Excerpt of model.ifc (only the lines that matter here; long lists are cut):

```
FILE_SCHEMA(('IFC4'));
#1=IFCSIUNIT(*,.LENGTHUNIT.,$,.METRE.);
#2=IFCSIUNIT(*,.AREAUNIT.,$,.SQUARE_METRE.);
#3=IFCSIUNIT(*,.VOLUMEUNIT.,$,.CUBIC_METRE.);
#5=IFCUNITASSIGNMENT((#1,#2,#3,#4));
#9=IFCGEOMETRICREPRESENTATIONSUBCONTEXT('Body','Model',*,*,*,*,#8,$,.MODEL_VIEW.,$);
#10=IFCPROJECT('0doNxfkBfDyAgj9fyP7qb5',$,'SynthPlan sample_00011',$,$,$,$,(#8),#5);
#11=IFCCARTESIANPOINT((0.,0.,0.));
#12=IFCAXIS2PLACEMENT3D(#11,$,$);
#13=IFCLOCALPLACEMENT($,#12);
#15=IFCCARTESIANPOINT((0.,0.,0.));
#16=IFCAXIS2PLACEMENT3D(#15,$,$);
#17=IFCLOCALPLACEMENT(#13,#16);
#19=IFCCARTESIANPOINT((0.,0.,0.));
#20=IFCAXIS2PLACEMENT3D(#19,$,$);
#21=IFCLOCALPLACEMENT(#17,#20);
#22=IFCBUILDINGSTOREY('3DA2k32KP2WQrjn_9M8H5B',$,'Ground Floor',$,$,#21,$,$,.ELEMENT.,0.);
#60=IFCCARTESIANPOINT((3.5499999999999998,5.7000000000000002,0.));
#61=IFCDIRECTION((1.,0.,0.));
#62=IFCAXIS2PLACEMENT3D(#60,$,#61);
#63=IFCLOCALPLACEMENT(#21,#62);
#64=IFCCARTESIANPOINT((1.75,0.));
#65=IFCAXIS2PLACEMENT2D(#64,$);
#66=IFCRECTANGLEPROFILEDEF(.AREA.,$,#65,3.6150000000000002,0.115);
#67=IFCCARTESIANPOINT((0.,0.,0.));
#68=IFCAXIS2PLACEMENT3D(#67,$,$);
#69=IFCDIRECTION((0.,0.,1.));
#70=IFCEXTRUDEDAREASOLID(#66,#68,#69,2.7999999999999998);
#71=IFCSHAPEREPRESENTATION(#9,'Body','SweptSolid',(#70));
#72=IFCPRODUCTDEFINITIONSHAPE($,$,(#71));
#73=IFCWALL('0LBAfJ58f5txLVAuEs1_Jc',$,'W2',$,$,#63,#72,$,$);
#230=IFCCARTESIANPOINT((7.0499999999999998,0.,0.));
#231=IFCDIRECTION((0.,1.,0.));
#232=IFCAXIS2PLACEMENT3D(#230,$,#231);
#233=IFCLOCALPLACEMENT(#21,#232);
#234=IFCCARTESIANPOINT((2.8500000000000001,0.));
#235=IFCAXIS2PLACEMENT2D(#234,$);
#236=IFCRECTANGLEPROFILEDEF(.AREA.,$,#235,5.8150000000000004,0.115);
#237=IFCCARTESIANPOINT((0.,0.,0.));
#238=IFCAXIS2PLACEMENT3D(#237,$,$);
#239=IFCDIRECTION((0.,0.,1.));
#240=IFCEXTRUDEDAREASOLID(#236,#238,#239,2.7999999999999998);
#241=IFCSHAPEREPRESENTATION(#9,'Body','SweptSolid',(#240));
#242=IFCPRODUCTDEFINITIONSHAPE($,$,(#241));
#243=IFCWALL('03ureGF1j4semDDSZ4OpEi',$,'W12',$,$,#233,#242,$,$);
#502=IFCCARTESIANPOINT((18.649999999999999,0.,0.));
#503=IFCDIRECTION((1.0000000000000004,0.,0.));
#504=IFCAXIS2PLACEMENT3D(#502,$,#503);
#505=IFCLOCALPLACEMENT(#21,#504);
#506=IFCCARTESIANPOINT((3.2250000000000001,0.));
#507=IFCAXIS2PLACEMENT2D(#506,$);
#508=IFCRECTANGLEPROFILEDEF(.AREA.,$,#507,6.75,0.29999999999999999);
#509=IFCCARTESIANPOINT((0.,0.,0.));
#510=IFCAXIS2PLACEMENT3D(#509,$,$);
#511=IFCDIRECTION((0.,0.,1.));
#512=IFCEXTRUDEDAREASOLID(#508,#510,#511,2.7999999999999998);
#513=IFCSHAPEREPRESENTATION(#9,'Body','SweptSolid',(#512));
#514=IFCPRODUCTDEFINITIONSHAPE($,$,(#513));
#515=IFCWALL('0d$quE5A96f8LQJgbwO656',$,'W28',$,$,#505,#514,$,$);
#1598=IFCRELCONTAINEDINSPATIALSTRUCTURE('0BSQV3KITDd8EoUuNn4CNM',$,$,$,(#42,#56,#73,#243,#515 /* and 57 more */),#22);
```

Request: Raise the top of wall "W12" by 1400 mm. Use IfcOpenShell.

```python
import ifcopenshell
import ifcopenshell.geom
import ifcopenshell.util.representation
import ifcopenshell.util.shape
import ifcopenshell.util.unit

model = ifcopenshell.open("model.ifc")
unit_scale = ifcopenshell.util.unit.calculate_unit_scale(model)
settings = ifcopenshell.geom.settings()


def volume(element):
    """Net volume in cubic metres, openings subtracted."""
    shape = ifcopenshell.geom.create_shape(settings, element)
    return ifcopenshell.util.shape.get_volume(shape.geometry)


wall = model.by_id(243)
before = volume(wall)

body = ifcopenshell.util.representation.get_representation(wall, "Model", "Body")
solid = body.Items[0]
old_height = solid.Depth
solid.Depth += 1.4 / unit_scale
after = volume(wall)

print(f"height {old_height:g} -> {solid.Depth:g}, volume {before:.3f} -> {after:.3f} m3")

model.write("model_updated.ifc")
```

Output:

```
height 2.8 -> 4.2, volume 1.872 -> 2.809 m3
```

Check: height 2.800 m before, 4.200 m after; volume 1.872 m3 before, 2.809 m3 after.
